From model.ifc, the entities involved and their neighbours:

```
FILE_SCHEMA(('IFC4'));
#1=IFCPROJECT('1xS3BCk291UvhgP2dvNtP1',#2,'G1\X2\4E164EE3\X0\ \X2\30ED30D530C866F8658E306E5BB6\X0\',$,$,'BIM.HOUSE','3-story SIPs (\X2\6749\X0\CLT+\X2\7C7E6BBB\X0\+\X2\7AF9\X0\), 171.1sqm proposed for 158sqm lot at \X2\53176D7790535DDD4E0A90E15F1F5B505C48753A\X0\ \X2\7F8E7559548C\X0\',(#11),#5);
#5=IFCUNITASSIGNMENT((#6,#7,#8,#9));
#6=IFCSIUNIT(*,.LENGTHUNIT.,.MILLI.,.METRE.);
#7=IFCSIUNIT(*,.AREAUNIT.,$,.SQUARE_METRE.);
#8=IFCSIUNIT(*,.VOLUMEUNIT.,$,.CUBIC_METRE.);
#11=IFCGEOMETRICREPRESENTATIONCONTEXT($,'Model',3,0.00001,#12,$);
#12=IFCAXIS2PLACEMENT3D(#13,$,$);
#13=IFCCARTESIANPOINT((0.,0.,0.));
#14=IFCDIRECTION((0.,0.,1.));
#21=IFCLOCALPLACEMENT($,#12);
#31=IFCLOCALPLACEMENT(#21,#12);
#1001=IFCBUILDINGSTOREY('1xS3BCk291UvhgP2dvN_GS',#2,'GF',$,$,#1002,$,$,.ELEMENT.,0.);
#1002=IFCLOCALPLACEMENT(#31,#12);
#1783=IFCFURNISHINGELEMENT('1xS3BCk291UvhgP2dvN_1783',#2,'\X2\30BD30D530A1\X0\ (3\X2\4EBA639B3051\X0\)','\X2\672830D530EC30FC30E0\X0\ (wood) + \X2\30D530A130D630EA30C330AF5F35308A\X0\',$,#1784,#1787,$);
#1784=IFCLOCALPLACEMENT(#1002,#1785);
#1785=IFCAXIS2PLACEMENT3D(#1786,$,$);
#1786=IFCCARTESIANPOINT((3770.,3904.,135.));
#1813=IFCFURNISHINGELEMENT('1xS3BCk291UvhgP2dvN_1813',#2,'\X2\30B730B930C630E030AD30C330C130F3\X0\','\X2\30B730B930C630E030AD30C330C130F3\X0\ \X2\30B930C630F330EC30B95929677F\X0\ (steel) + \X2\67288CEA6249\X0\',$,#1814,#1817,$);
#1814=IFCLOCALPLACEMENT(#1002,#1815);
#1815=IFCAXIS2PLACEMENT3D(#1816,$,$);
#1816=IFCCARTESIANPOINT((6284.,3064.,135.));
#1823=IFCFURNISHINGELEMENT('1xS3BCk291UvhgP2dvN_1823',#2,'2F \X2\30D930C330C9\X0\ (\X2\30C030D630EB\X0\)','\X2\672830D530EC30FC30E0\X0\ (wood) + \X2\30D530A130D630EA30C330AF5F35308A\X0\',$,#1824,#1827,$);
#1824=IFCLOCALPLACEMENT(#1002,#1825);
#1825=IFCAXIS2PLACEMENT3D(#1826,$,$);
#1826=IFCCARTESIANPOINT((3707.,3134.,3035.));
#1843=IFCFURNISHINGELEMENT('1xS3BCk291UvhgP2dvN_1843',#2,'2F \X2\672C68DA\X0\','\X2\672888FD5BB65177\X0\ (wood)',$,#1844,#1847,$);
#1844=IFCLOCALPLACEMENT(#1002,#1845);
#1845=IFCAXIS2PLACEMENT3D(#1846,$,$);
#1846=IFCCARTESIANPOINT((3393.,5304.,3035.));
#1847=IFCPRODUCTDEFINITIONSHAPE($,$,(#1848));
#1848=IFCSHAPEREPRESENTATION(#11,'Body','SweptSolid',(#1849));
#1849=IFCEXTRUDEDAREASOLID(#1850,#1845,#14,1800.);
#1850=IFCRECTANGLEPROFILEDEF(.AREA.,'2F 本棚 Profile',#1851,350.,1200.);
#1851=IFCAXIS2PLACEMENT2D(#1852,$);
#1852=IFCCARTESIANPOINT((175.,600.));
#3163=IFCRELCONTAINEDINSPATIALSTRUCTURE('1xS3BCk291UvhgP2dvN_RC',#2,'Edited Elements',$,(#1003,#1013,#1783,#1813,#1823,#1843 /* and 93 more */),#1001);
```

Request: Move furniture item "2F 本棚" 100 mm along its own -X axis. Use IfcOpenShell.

```python
import ifcopenshell
import ifcopenshell.api.geometry
import ifcopenshell.util.placement
import ifcopenshell.util.unit

model = ifcopenshell.open("model.ifc")
unit_scale = ifcopenshell.util.unit.calculate_unit_scale(model)

item = model.by_id(1843)
matrix = ifcopenshell.util.placement.get_local_placement(item.ObjectPlacement)
matrix[:3, 3] -= matrix[:3, 0] * 0.1 / unit_scale
ifcopenshell.api.geometry.edit_object_placement(model, product=item, matrix=matrix, is_si=False)

print(ifcopenshell.util.placement.get_local_placement(item.ObjectPlacement).round(3) + 0.0)

model.write("model_updated.ifc")
```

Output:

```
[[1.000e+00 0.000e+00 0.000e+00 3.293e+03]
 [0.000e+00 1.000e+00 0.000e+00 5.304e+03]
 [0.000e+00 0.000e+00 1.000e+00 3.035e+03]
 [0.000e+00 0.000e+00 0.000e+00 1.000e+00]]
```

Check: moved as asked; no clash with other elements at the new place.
